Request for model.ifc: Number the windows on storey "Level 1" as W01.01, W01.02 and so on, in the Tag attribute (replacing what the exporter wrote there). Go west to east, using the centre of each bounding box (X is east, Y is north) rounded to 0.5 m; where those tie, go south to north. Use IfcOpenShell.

First a look at what the model holds.

```python
import ifcopenshell
import ifcopenshell.util.element
import ifcopenshell.util.placement

model = ifcopenshell.open("model.ifc")
print(model.schema)
storey = next(s for s in model.by_type("IfcBuildingStorey") if s.Name == "Level 1")
windows = [e for e in ifcopenshell.util.element.get_decomposition(storey) if e.is_a("IfcWindow")]
for e in sorted(windows, key=lambda e: e.id()):
    origin = ifcopenshell.util.placement.get_local_placement(e.ObjectPlacement)[:3, 3]
    print(e.id(), e.Tag, e.Name, origin.round(2) + 0.0, sep=" | ")
```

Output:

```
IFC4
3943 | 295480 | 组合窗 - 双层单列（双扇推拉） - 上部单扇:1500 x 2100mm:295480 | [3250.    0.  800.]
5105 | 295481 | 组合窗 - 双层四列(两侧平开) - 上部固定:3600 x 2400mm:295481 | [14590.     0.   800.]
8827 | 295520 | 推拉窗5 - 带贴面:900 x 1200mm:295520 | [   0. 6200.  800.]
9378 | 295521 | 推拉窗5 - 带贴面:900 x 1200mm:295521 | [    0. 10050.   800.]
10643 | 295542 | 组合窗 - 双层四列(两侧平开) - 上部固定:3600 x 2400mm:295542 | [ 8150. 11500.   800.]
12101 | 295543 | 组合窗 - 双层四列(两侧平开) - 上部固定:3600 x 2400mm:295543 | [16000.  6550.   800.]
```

```python
import ifcopenshell
import ifcopenshell.geom
import ifcopenshell.util.element
import ifcopenshell.util.shape

model = ifcopenshell.open("model.ifc")
settings = ifcopenshell.geom.settings()
settings.set("use-world-coords", True)


def centre(element):
    shape = ifcopenshell.geom.create_shape(settings, element)
    return ifcopenshell.util.shape.get_bbox_centroid(shape.geometry)


storey = next(s for s in model.by_type("IfcBuildingStorey") if s.Name == "Level 1")
windows = [e for e in ifcopenshell.util.element.get_decomposition(storey) if e.is_a("IfcWindow")]

# Insertion points can sit at a corner or the storey origin, so sort by the geometry (in metres).
centres = {e: centre(e) for e in windows}
windows.sort(key=lambda e: (round(centres[e][0] / 0.5), centres[e][1]))

for i, e in enumerate(windows, start=1):
    number = f"W01.{i:02d}"
    e.Tag = number
    print(e.id(), number)

model.write("model-out.ifc")
```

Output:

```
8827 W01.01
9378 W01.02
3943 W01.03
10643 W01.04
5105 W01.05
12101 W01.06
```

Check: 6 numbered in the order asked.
